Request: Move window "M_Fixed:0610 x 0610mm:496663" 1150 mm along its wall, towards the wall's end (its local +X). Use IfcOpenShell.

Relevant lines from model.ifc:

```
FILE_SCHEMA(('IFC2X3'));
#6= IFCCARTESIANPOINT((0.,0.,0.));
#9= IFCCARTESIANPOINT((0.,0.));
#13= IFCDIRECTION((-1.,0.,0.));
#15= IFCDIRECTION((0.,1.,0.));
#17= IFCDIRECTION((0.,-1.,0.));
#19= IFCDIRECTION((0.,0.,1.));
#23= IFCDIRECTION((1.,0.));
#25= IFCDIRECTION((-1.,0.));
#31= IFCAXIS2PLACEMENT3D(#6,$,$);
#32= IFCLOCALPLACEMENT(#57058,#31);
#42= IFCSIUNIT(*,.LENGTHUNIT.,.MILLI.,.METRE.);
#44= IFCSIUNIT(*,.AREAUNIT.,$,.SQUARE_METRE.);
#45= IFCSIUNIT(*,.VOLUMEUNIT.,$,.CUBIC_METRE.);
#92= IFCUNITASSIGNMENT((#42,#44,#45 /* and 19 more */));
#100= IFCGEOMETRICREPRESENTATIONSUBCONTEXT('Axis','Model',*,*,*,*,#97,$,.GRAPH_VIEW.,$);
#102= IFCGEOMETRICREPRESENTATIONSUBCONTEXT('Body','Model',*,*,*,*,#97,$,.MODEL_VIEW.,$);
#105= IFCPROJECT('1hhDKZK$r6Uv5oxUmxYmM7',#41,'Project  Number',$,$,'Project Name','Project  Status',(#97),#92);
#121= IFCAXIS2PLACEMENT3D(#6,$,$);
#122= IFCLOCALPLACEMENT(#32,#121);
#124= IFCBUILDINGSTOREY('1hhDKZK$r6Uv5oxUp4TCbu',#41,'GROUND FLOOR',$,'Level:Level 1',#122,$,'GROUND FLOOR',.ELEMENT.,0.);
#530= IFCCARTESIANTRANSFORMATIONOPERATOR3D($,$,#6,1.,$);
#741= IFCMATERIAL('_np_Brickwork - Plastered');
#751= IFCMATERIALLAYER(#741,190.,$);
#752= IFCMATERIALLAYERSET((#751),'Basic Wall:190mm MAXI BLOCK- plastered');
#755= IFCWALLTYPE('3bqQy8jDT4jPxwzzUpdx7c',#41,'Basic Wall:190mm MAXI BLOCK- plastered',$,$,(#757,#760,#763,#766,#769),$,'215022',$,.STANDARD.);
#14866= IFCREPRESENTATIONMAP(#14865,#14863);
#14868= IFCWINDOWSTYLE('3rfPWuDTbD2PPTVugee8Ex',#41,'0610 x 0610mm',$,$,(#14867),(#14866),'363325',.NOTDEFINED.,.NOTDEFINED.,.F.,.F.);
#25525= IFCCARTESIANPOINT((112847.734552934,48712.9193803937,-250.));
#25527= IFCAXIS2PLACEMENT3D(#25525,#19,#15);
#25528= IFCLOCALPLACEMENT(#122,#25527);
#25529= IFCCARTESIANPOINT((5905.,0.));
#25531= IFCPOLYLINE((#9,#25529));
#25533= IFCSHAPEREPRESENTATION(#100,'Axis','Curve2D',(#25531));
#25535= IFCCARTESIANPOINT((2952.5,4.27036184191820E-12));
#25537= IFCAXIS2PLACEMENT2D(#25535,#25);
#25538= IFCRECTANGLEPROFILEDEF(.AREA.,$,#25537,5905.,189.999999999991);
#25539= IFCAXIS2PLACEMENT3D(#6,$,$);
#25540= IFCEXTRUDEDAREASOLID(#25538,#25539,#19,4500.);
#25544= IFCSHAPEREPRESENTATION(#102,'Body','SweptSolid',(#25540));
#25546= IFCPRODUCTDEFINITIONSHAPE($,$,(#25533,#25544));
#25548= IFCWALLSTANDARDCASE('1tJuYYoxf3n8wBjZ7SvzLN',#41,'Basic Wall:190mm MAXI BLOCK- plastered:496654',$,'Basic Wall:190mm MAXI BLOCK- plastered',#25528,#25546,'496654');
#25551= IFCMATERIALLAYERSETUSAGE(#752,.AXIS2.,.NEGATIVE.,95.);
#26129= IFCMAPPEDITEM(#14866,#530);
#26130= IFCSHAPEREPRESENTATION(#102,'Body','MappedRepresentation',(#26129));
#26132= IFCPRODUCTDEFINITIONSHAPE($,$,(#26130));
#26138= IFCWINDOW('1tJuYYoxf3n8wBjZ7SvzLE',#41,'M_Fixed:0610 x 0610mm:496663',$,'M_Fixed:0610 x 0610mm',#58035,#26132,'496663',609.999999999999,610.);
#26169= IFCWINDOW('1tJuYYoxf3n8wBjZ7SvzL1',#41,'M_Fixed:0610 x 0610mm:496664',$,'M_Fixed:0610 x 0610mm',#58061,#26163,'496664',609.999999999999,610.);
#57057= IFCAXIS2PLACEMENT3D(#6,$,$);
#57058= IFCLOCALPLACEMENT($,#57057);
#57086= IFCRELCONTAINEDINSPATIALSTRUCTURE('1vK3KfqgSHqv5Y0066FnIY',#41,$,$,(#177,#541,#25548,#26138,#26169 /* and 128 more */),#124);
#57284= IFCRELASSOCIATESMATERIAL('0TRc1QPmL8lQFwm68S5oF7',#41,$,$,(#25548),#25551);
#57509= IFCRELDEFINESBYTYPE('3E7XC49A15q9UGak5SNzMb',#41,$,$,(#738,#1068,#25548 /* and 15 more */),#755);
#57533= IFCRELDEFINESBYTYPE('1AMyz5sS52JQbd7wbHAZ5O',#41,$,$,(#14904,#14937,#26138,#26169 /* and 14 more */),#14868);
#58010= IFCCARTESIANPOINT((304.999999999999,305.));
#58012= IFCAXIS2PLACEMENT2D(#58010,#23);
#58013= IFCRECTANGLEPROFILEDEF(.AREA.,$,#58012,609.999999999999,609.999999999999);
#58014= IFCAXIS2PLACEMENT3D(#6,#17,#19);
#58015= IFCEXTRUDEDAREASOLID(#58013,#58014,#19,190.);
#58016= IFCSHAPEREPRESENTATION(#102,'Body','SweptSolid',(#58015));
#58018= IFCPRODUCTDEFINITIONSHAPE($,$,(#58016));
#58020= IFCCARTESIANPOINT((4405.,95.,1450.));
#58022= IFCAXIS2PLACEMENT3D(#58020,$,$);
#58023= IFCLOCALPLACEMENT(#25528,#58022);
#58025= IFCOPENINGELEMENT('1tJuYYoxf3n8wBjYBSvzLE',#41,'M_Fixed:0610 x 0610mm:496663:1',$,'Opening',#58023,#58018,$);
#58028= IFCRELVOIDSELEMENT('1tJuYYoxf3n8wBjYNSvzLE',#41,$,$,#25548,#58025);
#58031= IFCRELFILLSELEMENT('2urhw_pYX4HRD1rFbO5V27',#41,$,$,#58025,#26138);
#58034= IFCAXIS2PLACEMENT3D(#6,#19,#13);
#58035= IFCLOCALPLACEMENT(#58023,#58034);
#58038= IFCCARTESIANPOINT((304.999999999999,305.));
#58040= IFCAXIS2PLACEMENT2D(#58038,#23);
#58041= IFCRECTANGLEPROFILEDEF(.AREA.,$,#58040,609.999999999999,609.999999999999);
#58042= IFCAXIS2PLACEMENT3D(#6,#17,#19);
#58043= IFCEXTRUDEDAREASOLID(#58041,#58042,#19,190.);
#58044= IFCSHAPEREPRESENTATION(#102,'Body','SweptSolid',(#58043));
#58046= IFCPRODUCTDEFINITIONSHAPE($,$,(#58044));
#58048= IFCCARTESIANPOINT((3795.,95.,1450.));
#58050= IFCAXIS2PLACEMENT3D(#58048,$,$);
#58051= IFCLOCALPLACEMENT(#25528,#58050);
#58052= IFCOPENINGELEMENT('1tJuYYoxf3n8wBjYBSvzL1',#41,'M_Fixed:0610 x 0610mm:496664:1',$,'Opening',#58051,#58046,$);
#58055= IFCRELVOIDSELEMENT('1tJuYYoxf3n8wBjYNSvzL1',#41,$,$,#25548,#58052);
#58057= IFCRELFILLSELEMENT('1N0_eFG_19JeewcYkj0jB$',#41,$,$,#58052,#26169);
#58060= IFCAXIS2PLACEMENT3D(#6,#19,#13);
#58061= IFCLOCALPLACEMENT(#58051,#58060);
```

```python
import ifcopenshell
import ifcopenshell.api.geometry
import ifcopenshell.util.placement
import ifcopenshell.util.unit

model = ifcopenshell.open("model.ifc")
unit_scale = ifcopenshell.util.unit.calculate_unit_scale(model)

window = model.by_id(26138)
opening = window.FillsVoids[0].RelatingOpeningElement
wall = opening.VoidsElements[0].RelatingBuildingElement

wall_matrix = ifcopenshell.util.placement.get_local_placement(wall.ObjectPlacement)
shift = wall_matrix[:3, 0] * 1.15 / unit_scale
before = ifcopenshell.util.placement.get_local_placement(window.ObjectPlacement)[:3, 3].copy()

# The window is placed relative to its opening, so it follows when the opening moves.
matrix = ifcopenshell.util.placement.get_local_placement(opening.ObjectPlacement)
matrix[:3, 3] += shift
ifcopenshell.api.geometry.edit_object_placement(
    model, product=opening, matrix=matrix, is_si=False, should_transform_children=True
)

after = ifcopenshell.util.placement.get_local_placement(window.ObjectPlacement)[:3, 3]
print("window moved by", (after - before).round(3) + 0.0)

model.write("model_updated.ifc")
```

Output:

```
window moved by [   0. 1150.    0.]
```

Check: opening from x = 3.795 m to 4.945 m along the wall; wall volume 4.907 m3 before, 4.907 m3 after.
